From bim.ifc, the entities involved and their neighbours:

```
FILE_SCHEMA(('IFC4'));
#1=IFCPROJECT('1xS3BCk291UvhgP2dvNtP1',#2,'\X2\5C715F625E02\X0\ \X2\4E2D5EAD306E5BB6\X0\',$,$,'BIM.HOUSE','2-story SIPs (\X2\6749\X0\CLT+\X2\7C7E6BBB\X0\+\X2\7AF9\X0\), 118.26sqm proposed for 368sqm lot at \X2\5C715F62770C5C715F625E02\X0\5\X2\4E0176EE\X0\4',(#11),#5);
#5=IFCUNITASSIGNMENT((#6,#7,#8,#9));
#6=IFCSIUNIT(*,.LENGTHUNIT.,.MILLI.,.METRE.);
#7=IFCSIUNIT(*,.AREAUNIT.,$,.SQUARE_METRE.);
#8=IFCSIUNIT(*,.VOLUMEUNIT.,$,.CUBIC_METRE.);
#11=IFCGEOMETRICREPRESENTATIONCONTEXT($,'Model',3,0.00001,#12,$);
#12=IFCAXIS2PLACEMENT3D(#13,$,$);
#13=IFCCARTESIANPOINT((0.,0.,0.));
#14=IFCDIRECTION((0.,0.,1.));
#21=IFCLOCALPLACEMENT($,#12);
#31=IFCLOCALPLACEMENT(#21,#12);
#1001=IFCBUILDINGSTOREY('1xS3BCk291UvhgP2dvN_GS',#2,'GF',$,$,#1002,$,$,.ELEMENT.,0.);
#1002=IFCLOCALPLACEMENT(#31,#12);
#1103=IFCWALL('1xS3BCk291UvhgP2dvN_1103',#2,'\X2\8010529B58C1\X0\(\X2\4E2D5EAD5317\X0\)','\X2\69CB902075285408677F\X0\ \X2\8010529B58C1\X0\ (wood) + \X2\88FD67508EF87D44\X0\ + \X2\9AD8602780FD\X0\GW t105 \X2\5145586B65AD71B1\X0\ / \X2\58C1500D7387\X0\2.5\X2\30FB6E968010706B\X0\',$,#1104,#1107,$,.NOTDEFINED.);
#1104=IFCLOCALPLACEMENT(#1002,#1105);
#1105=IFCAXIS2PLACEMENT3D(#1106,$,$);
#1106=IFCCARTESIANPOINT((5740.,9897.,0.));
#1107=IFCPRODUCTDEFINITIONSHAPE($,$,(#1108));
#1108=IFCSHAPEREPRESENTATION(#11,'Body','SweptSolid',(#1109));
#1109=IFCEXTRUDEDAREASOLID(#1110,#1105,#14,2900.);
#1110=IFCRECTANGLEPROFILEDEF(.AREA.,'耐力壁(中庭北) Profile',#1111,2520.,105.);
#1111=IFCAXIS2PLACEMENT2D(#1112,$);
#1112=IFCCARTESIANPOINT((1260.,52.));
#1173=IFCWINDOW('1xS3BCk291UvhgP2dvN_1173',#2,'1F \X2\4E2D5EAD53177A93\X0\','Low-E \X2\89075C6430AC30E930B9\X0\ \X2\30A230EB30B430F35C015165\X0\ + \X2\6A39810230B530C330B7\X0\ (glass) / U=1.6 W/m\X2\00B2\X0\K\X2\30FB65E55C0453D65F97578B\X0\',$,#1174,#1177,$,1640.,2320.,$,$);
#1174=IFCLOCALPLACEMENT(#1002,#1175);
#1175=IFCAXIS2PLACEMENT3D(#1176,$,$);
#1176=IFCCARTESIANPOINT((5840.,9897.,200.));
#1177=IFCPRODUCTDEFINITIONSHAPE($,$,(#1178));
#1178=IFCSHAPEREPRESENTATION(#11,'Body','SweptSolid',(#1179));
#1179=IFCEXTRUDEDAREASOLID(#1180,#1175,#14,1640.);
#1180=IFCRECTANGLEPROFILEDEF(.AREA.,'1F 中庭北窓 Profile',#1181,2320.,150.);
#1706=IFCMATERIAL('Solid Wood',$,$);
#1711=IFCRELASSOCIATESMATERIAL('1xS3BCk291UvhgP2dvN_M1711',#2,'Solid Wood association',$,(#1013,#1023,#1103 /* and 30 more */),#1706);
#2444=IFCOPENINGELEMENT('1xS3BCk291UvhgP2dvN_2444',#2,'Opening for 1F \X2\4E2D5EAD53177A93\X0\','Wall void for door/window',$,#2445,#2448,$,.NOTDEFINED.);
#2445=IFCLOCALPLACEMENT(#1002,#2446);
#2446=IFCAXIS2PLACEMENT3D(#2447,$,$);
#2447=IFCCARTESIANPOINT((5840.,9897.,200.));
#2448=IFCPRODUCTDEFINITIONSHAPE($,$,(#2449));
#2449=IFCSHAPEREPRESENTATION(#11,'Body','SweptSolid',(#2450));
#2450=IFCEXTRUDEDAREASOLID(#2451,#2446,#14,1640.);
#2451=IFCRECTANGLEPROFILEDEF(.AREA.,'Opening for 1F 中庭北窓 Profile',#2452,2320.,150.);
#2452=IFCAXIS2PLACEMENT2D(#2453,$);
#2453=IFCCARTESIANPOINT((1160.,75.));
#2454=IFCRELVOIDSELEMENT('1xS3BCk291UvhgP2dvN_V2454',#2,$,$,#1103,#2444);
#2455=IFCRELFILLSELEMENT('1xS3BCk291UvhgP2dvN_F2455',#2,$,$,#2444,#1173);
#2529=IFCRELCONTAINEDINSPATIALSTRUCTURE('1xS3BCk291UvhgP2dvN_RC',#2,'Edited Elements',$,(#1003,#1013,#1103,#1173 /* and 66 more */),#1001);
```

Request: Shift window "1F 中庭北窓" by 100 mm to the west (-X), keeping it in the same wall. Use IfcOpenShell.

```python
import ifcopenshell
import ifcopenshell.api.geometry
import ifcopenshell.util.placement

model = ifcopenshell.open("bim.ifc")

window = model.by_guid("1xS3BCk291UvhgP2dvN_1173")
opening = window.FillsVoids[0].RelatingOpeningElement
wall = opening.VoidsElements[0].RelatingBuildingElement

wall_matrix = ifcopenshell.util.placement.get_local_placement(wall.ObjectPlacement)
shift = wall_matrix[:3, 0] * -100.0
before = ifcopenshell.util.placement.get_local_placement(window.ObjectPlacement)[:3, 3].copy()

# The window is not placed relative to its opening, so move both.
for product in (opening, window):
    matrix = ifcopenshell.util.placement.get_local_placement(product.ObjectPlacement)
    matrix[:3, 3] += shift
    ifcopenshell.api.geometry.edit_object_placement(model, product=product, matrix=matrix, is_si=False)

after = ifcopenshell.util.placement.get_local_placement(window.ObjectPlacement)[:3, 3]
print("window moved by", (after - before).round(3) + 0.0)

model.write("bim_rev.ifc")
```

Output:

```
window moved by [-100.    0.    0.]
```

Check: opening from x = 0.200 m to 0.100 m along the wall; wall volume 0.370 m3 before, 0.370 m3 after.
